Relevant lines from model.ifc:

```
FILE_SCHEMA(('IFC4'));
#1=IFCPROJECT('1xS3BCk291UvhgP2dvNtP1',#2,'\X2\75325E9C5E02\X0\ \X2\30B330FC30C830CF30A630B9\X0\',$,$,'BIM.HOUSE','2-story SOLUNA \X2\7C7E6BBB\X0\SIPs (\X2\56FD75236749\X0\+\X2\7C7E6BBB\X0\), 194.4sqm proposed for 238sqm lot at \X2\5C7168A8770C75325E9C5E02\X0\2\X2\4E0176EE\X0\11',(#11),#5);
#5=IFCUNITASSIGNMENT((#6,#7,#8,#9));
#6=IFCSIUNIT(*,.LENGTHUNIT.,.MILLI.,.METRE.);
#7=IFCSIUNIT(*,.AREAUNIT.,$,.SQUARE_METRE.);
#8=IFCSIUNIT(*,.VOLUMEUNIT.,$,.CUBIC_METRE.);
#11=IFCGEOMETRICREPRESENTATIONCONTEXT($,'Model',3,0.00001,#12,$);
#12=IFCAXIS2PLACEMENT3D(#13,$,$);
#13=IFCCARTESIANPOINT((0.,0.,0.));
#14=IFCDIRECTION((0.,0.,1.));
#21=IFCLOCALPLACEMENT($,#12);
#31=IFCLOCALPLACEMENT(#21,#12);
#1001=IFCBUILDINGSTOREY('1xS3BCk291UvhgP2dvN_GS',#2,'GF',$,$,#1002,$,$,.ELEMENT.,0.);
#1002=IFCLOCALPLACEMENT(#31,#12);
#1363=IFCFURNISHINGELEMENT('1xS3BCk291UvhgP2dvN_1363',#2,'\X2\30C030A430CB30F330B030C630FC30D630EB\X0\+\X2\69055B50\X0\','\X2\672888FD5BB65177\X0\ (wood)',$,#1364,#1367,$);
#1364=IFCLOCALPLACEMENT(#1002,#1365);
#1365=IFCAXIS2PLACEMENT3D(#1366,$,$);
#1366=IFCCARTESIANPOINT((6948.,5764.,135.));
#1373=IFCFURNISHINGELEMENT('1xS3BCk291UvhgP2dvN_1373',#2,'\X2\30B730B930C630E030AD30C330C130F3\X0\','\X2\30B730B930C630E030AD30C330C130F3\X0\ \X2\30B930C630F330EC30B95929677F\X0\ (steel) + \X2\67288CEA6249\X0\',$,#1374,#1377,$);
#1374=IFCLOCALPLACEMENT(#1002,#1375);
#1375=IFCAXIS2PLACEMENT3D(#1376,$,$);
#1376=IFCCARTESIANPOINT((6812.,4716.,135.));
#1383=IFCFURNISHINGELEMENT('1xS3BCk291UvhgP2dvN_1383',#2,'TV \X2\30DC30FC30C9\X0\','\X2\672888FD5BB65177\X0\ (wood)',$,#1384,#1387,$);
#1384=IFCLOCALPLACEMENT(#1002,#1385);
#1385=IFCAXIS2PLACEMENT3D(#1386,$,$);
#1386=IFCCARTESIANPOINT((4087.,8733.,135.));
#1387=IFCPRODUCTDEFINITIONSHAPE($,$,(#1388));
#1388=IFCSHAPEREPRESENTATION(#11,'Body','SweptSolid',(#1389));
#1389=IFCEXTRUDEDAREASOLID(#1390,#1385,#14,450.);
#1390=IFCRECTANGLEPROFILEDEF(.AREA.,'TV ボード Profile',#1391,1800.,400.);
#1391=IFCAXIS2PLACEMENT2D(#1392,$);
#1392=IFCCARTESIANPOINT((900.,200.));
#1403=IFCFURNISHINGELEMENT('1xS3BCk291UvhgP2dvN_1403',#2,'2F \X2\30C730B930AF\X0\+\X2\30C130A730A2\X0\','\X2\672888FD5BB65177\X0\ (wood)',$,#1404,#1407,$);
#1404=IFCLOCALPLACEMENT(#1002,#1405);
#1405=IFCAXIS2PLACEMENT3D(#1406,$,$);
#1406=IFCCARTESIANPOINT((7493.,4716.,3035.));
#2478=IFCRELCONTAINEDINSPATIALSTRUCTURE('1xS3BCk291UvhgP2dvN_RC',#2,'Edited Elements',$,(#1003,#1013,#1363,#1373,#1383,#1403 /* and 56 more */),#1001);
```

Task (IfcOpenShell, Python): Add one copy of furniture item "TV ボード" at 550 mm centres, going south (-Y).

```python
import numpy as np
import ifcopenshell
import ifcopenshell.api.geometry
import ifcopenshell.api.root
import ifcopenshell.util.element
import ifcopenshell.util.placement

model = ifcopenshell.open("model.ifc")


def reuse_history(source, copy):
    """copy_class also copies each property set's owner history, people and application; keep the originals."""
    for rel in copy.IsDefinedBy:
        if rel.is_a("IfcRelDefinesByProperties") and (history := rel.RelatingPropertyDefinition.OwnerHistory):
            rel.RelatingPropertyDefinition.OwnerHistory = source.OwnerHistory
            ifcopenshell.util.element.remove_deep2(model, history)


source = model.by_id(1383)
base = ifcopenshell.util.placement.get_local_placement(source.ObjectPlacement)
step = np.array([0.0, -1.0, 0.0]) * 550.0

for i in range(1, 2):
    copy = ifcopenshell.api.root.copy_class(model, product=source)
    copy.Representation = ifcopenshell.util.element.copy_deep(
        model, source.Representation, exclude=["IfcGeometricRepresentationContext", "IfcRepresentationMap"]
    )
    reuse_history(source, copy)
    matrix = base.copy()
    matrix[:3, 3] += i * step
    print("added at", matrix[:3, 3].round(3) + 0.0)
    ifcopenshell.api.geometry.edit_object_placement(model, product=copy, matrix=matrix, is_si=False)

model.write("model_v2.ifc")
```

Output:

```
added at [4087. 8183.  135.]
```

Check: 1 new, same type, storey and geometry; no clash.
